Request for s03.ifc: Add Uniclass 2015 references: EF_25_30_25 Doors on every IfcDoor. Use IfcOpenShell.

First a look at what the model holds.

```python
import ifcopenshell

model = ifcopenshell.open("s03.ifc")
print(model.schema)
print("classifications:", [c.Name for c in model.by_type("IfcClassification")])
for ifc_class in ("IfcDoor", "IfcRoof", "IfcStair", "IfcWall", "IfcWindow"):
    print(ifc_class, len(model.by_type(ifc_class)))
```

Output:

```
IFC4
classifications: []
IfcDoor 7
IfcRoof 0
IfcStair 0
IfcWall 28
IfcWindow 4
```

```python
import ifcopenshell
import ifcopenshell.api.classification

model = ifcopenshell.open("s03.ifc")

system = ifcopenshell.api.classification.add_classification(model, classification="Uniclass 2015")

codes = {
    "IfcDoor": ("EF_25_30_25", "Doors"),
}
for ifc_class, (code, name) in codes.items():
    products = model.by_type(ifc_class)
    ifcopenshell.api.classification.add_reference(
        model, products=products, classification=system, identification=code, name=name
    )
    print(code, len(products))

model.write("s03-out.ifc")
```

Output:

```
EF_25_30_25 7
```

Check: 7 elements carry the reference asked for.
